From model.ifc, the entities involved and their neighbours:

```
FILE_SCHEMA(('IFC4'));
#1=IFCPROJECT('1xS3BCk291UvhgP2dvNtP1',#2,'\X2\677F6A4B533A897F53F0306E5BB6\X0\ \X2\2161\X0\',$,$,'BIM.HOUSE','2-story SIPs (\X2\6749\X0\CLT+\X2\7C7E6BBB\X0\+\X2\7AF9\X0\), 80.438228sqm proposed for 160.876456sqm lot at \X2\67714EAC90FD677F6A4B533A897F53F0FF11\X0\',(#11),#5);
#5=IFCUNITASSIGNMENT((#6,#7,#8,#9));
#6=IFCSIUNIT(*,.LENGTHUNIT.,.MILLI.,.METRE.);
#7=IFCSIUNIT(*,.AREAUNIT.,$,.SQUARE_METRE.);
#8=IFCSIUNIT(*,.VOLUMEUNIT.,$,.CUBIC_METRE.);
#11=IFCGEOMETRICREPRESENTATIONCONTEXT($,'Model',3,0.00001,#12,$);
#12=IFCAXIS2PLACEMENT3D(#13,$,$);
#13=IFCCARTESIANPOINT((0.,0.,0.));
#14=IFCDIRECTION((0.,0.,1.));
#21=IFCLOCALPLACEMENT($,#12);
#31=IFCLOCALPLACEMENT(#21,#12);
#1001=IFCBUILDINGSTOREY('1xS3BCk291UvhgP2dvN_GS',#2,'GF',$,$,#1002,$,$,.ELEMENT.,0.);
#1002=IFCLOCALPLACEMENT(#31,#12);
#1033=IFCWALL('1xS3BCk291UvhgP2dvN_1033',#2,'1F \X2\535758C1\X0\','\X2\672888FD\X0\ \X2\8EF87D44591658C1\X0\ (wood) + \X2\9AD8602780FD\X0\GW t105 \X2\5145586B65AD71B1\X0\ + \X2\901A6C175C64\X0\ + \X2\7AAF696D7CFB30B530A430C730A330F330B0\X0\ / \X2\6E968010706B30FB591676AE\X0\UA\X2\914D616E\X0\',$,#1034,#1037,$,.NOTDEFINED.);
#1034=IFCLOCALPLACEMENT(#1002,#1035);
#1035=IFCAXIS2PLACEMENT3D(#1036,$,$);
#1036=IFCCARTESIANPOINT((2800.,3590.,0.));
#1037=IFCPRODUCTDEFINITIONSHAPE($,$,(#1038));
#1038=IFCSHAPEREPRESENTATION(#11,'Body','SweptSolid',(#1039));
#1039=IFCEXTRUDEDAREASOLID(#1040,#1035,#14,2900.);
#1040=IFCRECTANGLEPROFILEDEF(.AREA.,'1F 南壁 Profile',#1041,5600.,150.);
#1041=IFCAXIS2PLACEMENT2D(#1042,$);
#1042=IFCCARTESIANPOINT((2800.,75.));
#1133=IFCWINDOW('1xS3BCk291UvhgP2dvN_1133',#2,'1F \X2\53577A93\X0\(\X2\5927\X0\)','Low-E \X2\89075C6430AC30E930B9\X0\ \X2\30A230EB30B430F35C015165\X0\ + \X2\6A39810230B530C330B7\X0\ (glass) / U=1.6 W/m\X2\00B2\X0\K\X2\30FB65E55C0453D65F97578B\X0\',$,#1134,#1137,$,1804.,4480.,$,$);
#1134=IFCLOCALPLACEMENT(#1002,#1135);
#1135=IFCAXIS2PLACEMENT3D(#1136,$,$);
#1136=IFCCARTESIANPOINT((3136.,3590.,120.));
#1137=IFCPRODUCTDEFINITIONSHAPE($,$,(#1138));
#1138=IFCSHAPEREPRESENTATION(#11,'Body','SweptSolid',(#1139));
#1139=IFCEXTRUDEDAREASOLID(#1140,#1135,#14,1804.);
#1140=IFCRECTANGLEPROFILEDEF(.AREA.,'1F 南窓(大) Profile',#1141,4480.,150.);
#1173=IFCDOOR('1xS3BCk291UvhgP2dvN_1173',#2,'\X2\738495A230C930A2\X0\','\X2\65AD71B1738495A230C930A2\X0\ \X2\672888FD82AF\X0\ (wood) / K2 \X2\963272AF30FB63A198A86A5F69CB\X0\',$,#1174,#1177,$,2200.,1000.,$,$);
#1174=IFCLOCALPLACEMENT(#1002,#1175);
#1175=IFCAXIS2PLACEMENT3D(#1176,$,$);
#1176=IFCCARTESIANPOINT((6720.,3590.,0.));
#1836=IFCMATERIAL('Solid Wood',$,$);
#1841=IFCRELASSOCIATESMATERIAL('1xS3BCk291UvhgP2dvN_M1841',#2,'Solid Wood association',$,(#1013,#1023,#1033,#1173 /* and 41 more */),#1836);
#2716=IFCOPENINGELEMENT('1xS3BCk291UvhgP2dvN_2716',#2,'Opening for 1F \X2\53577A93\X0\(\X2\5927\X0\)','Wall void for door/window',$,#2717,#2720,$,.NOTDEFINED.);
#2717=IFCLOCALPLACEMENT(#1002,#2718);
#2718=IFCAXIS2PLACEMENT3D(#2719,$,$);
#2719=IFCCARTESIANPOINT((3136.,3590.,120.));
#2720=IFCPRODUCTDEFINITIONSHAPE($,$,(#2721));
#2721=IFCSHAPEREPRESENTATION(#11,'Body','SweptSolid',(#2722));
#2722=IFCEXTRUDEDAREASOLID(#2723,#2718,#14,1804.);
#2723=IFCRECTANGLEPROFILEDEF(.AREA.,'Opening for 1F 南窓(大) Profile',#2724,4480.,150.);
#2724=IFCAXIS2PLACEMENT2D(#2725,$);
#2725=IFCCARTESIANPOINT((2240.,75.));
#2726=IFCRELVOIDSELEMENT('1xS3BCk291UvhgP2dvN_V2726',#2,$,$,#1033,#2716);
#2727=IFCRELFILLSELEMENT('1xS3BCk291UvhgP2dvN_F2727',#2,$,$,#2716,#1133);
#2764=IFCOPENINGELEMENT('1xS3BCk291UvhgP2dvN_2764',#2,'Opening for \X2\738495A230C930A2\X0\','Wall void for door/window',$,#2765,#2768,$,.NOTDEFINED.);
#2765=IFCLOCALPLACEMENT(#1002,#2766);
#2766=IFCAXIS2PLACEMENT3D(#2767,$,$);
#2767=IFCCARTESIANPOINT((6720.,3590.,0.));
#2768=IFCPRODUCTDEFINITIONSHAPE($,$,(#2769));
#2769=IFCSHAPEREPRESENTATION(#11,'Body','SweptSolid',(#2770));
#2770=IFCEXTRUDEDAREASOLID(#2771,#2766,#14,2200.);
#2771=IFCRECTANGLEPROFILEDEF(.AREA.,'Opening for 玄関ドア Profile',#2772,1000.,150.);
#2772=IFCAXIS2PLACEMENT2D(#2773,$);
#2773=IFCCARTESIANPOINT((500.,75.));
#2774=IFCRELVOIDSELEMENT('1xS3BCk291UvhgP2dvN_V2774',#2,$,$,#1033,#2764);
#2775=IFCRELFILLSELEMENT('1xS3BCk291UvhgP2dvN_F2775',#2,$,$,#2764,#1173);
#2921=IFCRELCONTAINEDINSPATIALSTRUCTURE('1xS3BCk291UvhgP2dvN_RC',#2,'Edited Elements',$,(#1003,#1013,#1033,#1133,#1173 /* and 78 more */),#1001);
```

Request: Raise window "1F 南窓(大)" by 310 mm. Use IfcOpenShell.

```python
import numpy as np
import ifcopenshell
import ifcopenshell.api.geometry
import ifcopenshell.util.placement
import ifcopenshell.util.unit

model = ifcopenshell.open("model.ifc")
unit_scale = ifcopenshell.util.unit.calculate_unit_scale(model)

window = model.by_guid("1xS3BCk291UvhgP2dvN_1133")
opening = window.FillsVoids[0].RelatingOpeningElement
dz = 310.0

shift = np.array([0.0, 0.0, dz])
# The window is not placed relative to its opening, so move both.
for product in (opening, window):
    matrix = ifcopenshell.util.placement.get_local_placement(product.ObjectPlacement)
    matrix[:3, 3] += shift
    ifcopenshell.api.geometry.edit_object_placement(model, product=product, matrix=matrix, is_si=False)

print(f"moved by {dz * unit_scale:+.3f} m")

model.write("model_rev.ifc")
```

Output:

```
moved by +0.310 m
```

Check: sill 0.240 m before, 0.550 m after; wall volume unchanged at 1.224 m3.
